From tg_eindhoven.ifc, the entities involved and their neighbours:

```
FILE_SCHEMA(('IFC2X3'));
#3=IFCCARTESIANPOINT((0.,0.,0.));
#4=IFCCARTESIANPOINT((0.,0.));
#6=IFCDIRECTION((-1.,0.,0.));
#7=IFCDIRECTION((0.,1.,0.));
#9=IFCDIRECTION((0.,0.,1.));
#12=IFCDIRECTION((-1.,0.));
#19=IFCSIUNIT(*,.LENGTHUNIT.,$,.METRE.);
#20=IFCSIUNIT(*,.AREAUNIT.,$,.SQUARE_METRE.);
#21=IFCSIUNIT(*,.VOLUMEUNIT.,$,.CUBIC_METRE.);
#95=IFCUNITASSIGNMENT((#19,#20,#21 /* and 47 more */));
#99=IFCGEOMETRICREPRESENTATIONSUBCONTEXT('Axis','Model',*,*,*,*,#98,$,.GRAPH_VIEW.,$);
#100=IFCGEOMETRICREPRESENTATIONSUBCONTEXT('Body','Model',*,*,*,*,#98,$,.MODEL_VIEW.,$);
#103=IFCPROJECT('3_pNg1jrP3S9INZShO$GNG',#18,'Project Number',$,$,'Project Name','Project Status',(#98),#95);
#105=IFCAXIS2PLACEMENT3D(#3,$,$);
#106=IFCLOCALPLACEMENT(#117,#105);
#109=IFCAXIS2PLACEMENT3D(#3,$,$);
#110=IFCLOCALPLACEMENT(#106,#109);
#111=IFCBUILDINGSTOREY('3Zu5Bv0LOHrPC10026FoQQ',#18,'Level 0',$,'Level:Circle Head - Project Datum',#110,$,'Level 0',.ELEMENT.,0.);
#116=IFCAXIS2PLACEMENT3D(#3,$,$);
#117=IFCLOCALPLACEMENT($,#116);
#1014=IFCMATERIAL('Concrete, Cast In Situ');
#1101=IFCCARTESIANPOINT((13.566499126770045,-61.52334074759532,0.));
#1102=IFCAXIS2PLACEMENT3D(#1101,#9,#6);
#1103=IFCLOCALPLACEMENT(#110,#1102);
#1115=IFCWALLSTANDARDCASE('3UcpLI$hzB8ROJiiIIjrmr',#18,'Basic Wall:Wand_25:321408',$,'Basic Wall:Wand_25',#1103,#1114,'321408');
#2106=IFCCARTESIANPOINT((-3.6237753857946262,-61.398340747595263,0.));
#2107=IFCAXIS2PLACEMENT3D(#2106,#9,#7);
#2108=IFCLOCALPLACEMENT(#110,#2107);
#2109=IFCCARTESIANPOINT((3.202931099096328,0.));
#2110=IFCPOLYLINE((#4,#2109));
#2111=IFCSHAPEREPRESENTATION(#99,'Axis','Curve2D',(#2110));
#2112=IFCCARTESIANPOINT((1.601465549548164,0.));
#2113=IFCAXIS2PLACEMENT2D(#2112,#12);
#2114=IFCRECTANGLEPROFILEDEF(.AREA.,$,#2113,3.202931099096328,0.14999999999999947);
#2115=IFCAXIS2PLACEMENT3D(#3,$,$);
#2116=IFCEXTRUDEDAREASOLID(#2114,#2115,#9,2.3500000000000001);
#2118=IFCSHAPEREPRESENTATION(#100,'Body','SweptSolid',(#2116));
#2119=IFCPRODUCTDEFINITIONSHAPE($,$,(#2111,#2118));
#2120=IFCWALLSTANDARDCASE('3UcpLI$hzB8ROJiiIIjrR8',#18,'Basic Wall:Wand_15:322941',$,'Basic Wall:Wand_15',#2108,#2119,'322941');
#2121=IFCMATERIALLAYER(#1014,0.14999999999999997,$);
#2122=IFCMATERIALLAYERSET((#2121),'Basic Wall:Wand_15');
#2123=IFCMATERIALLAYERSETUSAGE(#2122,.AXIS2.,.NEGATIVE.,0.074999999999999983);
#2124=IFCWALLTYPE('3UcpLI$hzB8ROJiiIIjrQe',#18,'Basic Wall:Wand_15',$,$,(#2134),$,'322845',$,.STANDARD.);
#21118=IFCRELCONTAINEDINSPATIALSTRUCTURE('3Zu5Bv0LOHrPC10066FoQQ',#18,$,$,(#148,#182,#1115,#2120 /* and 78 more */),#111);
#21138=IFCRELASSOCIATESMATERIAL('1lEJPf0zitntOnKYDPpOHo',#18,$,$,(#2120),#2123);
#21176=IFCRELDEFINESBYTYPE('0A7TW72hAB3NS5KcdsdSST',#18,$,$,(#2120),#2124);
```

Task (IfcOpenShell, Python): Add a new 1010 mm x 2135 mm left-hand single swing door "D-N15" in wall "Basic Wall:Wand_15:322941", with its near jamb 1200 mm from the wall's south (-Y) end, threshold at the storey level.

```python
import numpy as np
import ifcopenshell
import ifcopenshell.api.feature
import ifcopenshell.api.geometry
import ifcopenshell.api.root
import ifcopenshell.api.spatial
import ifcopenshell.api.type
import ifcopenshell.geom
import ifcopenshell.util.element
import ifcopenshell.util.placement
import ifcopenshell.util.representation
import ifcopenshell.util.shape
import ifcopenshell.util.unit

model = ifcopenshell.open("tg_eindhoven.ifc")
unit_scale = ifcopenshell.util.unit.calculate_unit_scale(model)
settings = ifcopenshell.geom.settings()


def volume(element):
    """Net volume in cubic metres, openings subtracted."""
    shape = ifcopenshell.geom.create_shape(settings, element)
    return ifcopenshell.util.shape.get_volume(shape.geometry)


wall = model.by_id(2120)
storey = ifcopenshell.util.element.get_container(wall, ifc_class="IfcBuildingStorey")
context = ifcopenshell.util.representation.get_context(model, "Model", "Body", "MODEL_VIEW")
before = volume(wall)

width, height, from_end, sill = 1.01, 2.135, 1.2, 0.0  # metres

# The wall runs along its own X axis, and the end named is its -X end.
wall_shape = ifcopenshell.geom.create_shape(settings, wall)
x, y, z = ifcopenshell.util.shape.get_vertices(wall_shape.geometry).T
start = x.min() + from_end
face, thickness = float(y.min()), float(y.max() - y.min())
wall_matrix = ifcopenshell.util.placement.get_local_placement(wall.ObjectPlacement)
level = ifcopenshell.util.placement.get_local_placement(storey.ObjectPlacement)[2, 3]


def in_wall(x, y):
    """Placement at x, y metres in the wall's axes, at sill height."""
    matrix = wall_matrix.copy()
    matrix[:, 3] = wall_matrix @ np.array([x / unit_scale, y / unit_scale, 0.0, 1.0])
    matrix[2, 3] = level + sill / unit_scale
    return matrix


# Opening: a box that overshoots both wall faces by 50 mm.
opening = ifcopenshell.api.root.create_entity(model, ifc_class="IfcOpeningElement")
box = ifcopenshell.api.geometry.add_wall_representation(
    model, context=context, length=width, height=height, thickness=thickness + 0.1
)
ifcopenshell.api.geometry.assign_representation(model, product=opening, representation=box)
ifcopenshell.api.geometry.edit_object_placement(model, product=opening, matrix=in_wall(start, face - 0.05), is_si=False)
ifcopenshell.api.feature.add_feature(model, feature=opening, element=wall)

door = ifcopenshell.api.root.create_entity(model, ifc_class="IfcDoor", name="D-N15")
door.OverallWidth, door.OverallHeight = width / unit_scale, height / unit_scale
body = ifcopenshell.api.geometry.add_door_representation(
    model,
    context=context,
    overall_width=door.OverallWidth,
    overall_height=door.OverallHeight,
    operation_type="SINGLE_SWING_LEFT",
    lining_properties={"LiningDepth": thickness / unit_scale, "ThresholdDepth": thickness / unit_scale},
)
ifcopenshell.api.geometry.assign_representation(model, product=door, representation=body)
ifcopenshell.api.spatial.assign_container(model, products=[door], relating_structure=storey)
fills = ifcopenshell.api.feature.add_filling(model, opening=opening, element=door)
fills.OwnerHistory = door.OwnerHistory  # required in IFC2X3

# IFC2X3 keeps the operation on the door style.
style = ifcopenshell.api.root.create_entity(model, ifc_class="IfcDoorStyle", name="D-N15")
style.OperationType, style.ConstructionType = "SINGLE_SWING_LEFT", "NOTDEFINED"
style.ParameterTakesPrecedence = style.Sizeable = False
ifcopenshell.api.type.assign_type(model, related_objects=[door], relating_type=style)

# The lining spans the wall, so the door starts at the wall face.
ifcopenshell.api.geometry.edit_object_placement(model, product=door, matrix=in_wall(start, face), is_si=False)

after = volume(wall)

print(f"wall volume {before:.3f} -> {after:.3f} m3")

model.write("tg_eindhoven_edited.ifc")
```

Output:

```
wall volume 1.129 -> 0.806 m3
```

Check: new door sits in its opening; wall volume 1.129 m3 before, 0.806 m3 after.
